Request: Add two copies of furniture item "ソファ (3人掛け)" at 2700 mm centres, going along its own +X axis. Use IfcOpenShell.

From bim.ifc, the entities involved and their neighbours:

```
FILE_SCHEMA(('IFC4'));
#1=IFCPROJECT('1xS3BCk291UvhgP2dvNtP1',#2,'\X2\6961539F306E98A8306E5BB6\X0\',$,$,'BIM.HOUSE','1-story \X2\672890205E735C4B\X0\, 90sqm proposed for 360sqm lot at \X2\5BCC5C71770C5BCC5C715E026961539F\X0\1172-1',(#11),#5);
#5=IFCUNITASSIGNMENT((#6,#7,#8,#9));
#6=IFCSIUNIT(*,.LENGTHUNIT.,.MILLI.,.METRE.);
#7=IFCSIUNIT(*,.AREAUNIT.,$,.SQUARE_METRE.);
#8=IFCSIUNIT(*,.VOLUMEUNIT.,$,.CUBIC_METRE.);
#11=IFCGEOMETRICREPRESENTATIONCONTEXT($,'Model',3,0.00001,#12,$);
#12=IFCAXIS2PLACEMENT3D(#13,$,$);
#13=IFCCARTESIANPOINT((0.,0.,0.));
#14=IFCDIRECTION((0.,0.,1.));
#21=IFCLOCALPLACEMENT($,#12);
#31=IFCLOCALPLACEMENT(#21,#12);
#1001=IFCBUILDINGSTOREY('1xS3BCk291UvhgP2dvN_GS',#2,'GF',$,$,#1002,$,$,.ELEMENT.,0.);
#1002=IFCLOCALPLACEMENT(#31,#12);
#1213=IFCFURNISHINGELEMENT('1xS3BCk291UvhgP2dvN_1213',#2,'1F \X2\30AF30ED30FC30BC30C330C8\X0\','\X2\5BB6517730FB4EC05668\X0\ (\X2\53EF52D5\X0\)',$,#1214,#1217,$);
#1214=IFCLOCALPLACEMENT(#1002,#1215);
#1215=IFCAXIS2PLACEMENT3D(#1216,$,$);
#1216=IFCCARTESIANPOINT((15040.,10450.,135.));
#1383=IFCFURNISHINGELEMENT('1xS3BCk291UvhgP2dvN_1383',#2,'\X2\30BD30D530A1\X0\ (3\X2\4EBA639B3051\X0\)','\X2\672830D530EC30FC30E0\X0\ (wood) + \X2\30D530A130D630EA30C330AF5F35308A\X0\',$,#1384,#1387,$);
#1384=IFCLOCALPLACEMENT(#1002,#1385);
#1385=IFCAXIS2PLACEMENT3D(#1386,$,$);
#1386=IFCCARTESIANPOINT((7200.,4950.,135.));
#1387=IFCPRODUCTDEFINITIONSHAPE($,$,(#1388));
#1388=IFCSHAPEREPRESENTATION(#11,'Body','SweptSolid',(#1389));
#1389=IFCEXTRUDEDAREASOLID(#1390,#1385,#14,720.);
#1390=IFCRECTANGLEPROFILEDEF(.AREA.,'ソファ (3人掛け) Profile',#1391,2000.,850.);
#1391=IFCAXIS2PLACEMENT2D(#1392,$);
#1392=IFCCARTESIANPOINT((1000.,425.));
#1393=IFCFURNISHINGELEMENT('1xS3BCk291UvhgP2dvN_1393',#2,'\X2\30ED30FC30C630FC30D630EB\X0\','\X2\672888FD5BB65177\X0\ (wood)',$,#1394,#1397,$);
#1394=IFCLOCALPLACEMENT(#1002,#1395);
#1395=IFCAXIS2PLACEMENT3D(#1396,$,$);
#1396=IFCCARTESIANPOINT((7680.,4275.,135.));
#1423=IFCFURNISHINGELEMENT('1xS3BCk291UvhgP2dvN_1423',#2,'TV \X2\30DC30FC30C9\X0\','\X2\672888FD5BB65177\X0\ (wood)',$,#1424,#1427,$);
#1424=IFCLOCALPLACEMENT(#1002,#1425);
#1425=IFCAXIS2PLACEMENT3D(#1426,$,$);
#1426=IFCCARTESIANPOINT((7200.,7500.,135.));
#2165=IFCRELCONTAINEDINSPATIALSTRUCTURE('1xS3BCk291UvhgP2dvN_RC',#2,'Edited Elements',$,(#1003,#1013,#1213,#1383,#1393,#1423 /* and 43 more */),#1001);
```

```python
import ifcopenshell
import ifcopenshell.api.geometry
import ifcopenshell.api.root
import ifcopenshell.util.element
import ifcopenshell.util.placement
import ifcopenshell.util.unit

model = ifcopenshell.open("bim.ifc")
unit_scale = ifcopenshell.util.unit.calculate_unit_scale(model)


def reuse_history(source, copy):
    """copy_class also copies each property set's owner history, people and application; keep the originals."""
    for rel in copy.IsDefinedBy:
        if rel.is_a("IfcRelDefinesByProperties") and (history := rel.RelatingPropertyDefinition.OwnerHistory):
            rel.RelatingPropertyDefinition.OwnerHistory = source.OwnerHistory
            ifcopenshell.util.element.remove_deep2(model, history)


source = model.by_id(1383)
base = ifcopenshell.util.placement.get_local_placement(source.ObjectPlacement)
step = base[:3, 0] * 2.7 / unit_scale

for i in range(1, 3):
    copy = ifcopenshell.api.root.copy_class(model, product=source)
    copy.Representation = ifcopenshell.util.element.copy_deep(
        model, source.Representation, exclude=["IfcGeometricRepresentationContext", "IfcRepresentationMap"]
    )
    reuse_history(source, copy)
    matrix = base.copy()
    matrix[:3, 3] += i * step
    print("added at", matrix[:3, 3].round(3) + 0.0)
    ifcopenshell.api.geometry.edit_object_placement(model, product=copy, matrix=matrix, is_si=False)

model.write("bim_rev.ifc")
```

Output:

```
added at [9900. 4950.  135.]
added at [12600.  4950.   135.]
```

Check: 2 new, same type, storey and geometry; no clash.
